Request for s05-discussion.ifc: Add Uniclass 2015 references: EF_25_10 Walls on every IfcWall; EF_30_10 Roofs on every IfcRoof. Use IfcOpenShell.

First a look at what the model holds.

```python
import ifcopenshell

model = ifcopenshell.open("s05-discussion.ifc")
print(model.schema)
print("classifications:", [c.Name for c in model.by_type("IfcClassification")])
for ifc_class in ("IfcDoor", "IfcRoof", "IfcStair", "IfcWall", "IfcWindow"):
    print(ifc_class, len(model.by_type(ifc_class)))
```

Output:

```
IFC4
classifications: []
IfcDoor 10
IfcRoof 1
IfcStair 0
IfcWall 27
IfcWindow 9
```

```python
import ifcopenshell
import ifcopenshell.api.classification

model = ifcopenshell.open("s05-discussion.ifc")

system = ifcopenshell.api.classification.add_classification(model, classification="Uniclass 2015")

codes = {
    "IfcWall": ("EF_25_10", "Walls"),
    "IfcRoof": ("EF_30_10", "Roofs"),
}
for ifc_class, (code, name) in codes.items():
    products = model.by_type(ifc_class)
    ifcopenshell.api.classification.add_reference(
        model, products=products, classification=system, identification=code, name=name
    )
    print(code, len(products))

model.write("s05-discussion_v2.ifc")
```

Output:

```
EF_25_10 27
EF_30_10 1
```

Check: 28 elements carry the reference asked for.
